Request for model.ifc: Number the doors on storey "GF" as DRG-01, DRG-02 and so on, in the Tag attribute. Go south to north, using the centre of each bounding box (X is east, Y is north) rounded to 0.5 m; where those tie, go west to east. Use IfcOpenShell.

First a look at what the model holds.

```python
import ifcopenshell
import ifcopenshell.util.element
import ifcopenshell.util.placement

model = ifcopenshell.open("model.ifc")
print(model.schema)
storey = next(s for s in model.by_type("IfcBuildingStorey") if s.Name == "GF")
doors = [e for e in ifcopenshell.util.element.get_decomposition(storey) if e.is_a("IfcDoor")]
for e in sorted(doors, key=lambda e: e.id()):
    origin = ifcopenshell.util.placement.get_local_placement(e.ObjectPlacement)[:3, 3]
    print(e.id(), e.Tag, e.Name, origin.round(2) + 0.0, sep=" | ")
```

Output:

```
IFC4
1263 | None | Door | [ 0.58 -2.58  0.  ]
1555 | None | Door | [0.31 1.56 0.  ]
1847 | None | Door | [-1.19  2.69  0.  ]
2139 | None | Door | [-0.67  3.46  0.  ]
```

```python
import ifcopenshell
import ifcopenshell.geom
import ifcopenshell.util.element
import ifcopenshell.util.shape

model = ifcopenshell.open("model.ifc")
settings = ifcopenshell.geom.settings()
settings.set("use-world-coords", True)


def centre(element):
    shape = ifcopenshell.geom.create_shape(settings, element)
    return ifcopenshell.util.shape.get_bbox_centroid(shape.geometry)


storey = next(s for s in model.by_type("IfcBuildingStorey") if s.Name == "GF")
doors = [e for e in ifcopenshell.util.element.get_decomposition(storey) if e.is_a("IfcDoor")]

# Insertion points can sit at a corner or the storey origin, so sort by the geometry (in metres).
centres = {e: centre(e) for e in doors}
doors.sort(key=lambda e: (round(centres[e][1] / 0.5), centres[e][0]))

for i, e in enumerate(doors, start=1):
    number = f"DRG-{i:02d}"
    e.Tag = number
    print(e.id(), number)

model.write("model_v2.ifc")
```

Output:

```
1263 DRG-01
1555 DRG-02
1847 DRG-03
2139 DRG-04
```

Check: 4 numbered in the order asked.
